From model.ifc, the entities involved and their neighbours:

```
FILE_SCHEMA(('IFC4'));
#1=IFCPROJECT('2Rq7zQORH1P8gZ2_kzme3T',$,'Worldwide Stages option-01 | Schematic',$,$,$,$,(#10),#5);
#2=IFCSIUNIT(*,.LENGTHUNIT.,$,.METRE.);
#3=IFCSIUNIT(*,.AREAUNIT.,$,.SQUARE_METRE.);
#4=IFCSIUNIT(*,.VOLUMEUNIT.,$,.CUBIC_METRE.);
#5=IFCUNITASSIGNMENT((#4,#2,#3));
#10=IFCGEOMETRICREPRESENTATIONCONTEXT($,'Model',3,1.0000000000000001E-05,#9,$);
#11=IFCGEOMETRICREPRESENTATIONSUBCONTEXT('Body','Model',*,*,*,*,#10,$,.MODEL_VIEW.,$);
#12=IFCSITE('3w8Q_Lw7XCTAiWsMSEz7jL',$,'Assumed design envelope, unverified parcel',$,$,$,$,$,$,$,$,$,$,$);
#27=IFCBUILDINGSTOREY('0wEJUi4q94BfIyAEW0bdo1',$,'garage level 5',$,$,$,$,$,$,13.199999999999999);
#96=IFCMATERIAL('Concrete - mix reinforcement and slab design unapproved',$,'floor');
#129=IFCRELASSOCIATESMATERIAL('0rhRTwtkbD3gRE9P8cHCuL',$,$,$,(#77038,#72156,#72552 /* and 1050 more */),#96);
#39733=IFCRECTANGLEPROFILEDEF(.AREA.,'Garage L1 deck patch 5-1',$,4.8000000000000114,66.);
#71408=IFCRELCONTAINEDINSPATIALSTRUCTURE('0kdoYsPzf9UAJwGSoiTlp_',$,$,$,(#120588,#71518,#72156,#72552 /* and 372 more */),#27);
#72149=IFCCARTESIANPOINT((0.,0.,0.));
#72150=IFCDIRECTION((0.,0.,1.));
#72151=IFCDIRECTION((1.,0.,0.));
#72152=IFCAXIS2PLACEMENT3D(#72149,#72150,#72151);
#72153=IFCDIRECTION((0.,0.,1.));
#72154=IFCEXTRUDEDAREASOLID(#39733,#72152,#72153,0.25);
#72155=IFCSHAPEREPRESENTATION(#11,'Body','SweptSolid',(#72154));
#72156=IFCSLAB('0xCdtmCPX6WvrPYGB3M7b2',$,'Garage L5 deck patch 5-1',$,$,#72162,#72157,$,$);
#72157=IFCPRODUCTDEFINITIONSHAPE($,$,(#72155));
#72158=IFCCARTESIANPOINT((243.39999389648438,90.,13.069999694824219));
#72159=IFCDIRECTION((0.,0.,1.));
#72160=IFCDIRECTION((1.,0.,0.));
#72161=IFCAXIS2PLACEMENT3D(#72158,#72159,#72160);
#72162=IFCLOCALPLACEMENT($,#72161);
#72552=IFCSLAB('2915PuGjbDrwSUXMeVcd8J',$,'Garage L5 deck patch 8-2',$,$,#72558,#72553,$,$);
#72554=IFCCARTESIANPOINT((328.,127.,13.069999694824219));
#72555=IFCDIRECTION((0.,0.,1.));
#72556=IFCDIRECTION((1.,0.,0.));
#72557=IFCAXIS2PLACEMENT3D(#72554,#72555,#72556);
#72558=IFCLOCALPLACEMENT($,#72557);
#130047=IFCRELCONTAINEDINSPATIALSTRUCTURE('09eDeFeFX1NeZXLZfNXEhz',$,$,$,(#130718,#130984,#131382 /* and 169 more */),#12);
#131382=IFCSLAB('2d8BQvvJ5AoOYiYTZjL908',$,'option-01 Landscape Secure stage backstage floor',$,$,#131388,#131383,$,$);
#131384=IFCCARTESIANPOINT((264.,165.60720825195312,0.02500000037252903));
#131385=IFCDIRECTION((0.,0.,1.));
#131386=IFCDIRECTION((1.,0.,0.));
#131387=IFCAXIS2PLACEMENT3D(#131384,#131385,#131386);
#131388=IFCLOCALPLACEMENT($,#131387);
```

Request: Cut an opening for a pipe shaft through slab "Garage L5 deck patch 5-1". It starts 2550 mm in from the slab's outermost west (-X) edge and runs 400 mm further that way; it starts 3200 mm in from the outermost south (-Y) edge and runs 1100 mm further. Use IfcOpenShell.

```python
import numpy as np
import ifcopenshell
import ifcopenshell.api.feature
import ifcopenshell.api.geometry
import ifcopenshell.api.root
import ifcopenshell.geom
import ifcopenshell.util.placement
import ifcopenshell.util.representation
import ifcopenshell.util.shape
import ifcopenshell.util.unit

model = ifcopenshell.open("model.ifc")
unit_scale = ifcopenshell.util.unit.calculate_unit_scale(model)
settings = ifcopenshell.geom.settings()


def volume(element):
    """Net volume in cubic metres, openings subtracted."""
    shape = ifcopenshell.geom.create_shape(settings, element)
    return ifcopenshell.util.shape.get_volume(shape.geometry)


slab = model.by_id(72156)
before = volume(slab)

# Extent in the slab's own axes, in metres. The edges named are its -X and -Y sides.
slab_shape = ifcopenshell.geom.create_shape(settings, slab)
vertices = ifcopenshell.util.shape.get_vertices(slab_shape.geometry)
x_min, y_min, bottom = vertices.min(axis=0)
top = vertices[:, 2].max()

opening = ifcopenshell.api.root.create_entity(model, ifc_class="IfcOpeningElement", name="Pipe shaft opening", predefined_type="OPENING")
context = ifcopenshell.util.representation.get_context(model, "Model", "Body", "MODEL_VIEW")
width, depth = 0.4, 1.1
outline = [(0.0, 0.0), (width, 0.0), (width, depth), (0.0, depth), (0.0, 0.0)]
# Overshoot both faces by 50 mm so the cut is clean.
shape = ifcopenshell.api.geometry.add_slab_representation(
    model, context=context, depth=top - bottom + 0.1, polyline=outline
)
ifcopenshell.api.geometry.assign_representation(model, product=opening, representation=shape)

matrix = ifcopenshell.util.placement.get_local_placement(slab.ObjectPlacement)
matrix[:, 3] = matrix @ np.append(np.array([x_min + 2.55, y_min + 3.2, bottom - 0.05]) / unit_scale, 1.0)
ifcopenshell.api.geometry.edit_object_placement(model, product=opening, matrix=matrix, is_si=False)
ifcopenshell.api.feature.add_feature(model, feature=opening, element=slab)

after = volume(slab)

print(f"slab volume {before:.3f} -> {after:.3f} m3")

model.write("model_edited.ifc")
```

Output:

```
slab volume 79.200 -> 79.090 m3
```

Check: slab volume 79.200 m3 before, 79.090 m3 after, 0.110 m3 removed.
